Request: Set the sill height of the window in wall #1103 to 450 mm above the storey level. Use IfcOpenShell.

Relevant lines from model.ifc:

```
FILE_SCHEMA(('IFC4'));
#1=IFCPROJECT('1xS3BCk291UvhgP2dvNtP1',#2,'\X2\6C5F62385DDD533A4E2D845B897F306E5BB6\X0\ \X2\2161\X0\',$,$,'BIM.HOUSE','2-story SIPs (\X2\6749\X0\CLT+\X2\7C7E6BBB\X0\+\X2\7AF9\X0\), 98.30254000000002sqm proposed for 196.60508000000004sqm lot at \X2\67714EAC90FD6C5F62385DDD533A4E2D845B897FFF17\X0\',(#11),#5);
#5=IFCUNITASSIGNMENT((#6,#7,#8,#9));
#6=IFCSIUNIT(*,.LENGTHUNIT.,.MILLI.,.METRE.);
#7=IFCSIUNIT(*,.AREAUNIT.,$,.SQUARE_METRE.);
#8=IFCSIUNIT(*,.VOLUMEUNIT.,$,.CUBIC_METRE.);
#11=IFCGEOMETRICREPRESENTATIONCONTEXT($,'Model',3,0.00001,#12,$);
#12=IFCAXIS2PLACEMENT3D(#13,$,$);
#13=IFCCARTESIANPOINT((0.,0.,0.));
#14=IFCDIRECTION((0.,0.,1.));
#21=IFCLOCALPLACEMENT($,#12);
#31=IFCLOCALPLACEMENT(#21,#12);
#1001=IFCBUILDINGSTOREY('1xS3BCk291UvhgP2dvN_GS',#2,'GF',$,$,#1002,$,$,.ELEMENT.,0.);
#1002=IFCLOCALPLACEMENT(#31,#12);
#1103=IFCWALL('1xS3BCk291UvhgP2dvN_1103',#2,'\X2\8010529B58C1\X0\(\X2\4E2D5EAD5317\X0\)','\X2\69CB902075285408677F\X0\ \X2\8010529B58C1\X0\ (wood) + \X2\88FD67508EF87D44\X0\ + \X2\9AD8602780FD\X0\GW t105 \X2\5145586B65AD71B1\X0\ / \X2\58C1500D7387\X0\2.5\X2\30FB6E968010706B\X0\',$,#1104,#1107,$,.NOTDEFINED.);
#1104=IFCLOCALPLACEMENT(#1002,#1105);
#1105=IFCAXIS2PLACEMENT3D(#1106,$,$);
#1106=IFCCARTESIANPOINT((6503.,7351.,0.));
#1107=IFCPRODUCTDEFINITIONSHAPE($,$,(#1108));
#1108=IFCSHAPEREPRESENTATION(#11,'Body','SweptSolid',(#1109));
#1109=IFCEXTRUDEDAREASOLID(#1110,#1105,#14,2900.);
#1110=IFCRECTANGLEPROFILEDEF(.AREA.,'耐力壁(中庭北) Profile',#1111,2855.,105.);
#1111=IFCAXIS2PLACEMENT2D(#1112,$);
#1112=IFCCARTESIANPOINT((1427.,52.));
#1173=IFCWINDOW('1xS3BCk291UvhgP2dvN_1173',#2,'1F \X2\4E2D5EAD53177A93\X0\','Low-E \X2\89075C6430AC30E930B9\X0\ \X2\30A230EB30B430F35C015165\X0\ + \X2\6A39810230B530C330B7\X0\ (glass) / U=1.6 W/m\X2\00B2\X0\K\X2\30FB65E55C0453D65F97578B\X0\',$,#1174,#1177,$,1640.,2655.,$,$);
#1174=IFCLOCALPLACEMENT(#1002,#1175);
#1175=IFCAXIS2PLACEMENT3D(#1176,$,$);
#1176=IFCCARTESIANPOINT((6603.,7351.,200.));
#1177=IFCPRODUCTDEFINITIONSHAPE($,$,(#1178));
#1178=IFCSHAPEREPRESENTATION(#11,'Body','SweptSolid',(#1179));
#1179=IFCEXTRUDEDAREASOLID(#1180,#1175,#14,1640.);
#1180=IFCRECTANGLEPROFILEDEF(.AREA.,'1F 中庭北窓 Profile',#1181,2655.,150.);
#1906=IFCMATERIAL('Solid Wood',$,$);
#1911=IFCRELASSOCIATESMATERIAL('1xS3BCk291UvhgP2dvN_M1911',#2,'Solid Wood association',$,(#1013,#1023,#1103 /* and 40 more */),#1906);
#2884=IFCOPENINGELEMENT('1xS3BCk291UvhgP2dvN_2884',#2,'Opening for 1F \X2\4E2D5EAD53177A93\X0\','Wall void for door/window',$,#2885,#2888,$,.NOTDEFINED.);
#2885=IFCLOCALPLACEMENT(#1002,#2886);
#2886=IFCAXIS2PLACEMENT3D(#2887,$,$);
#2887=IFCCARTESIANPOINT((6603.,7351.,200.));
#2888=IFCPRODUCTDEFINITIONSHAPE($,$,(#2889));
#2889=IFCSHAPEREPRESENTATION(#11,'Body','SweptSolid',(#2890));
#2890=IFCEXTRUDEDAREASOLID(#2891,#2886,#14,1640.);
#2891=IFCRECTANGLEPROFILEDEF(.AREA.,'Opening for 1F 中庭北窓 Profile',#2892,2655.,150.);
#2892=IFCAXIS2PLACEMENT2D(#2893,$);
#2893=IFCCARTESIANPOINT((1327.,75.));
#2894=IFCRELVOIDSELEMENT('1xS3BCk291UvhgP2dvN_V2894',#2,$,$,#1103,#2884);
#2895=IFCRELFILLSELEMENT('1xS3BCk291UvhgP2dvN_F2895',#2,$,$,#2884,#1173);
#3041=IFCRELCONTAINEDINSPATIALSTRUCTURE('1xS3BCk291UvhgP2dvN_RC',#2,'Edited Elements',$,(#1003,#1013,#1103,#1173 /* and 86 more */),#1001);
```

```python
import numpy as np
import ifcopenshell
import ifcopenshell.api.geometry
import ifcopenshell.geom
import ifcopenshell.util.element
import ifcopenshell.util.placement
import ifcopenshell.util.shape
import ifcopenshell.util.unit

model = ifcopenshell.open("model.ifc")
unit_scale = ifcopenshell.util.unit.calculate_unit_scale(model)

window = model.by_guid("1xS3BCk291UvhgP2dvN_1173")
opening = window.FillsVoids[0].RelatingOpeningElement
storey = ifcopenshell.util.element.get_container(window, ifc_class="IfcBuildingStorey")
level = ifcopenshell.util.placement.get_local_placement(storey.ObjectPlacement)[2, 3]

# The opening's origin need not be at the sill, so measure its lowest point.
shape = ifcopenshell.geom.create_shape(ifcopenshell.geom.settings(), opening)
bottom = ifcopenshell.util.shape.get_shape_bottom_elevation(shape, shape.geometry) / unit_scale
dz = level + 0.45 / unit_scale - bottom

shift = np.array([0.0, 0.0, dz])
# The window is not placed relative to its opening, so move both.
for product in (opening, window):
    matrix = ifcopenshell.util.placement.get_local_placement(product.ObjectPlacement)
    matrix[:3, 3] += shift
    ifcopenshell.api.geometry.edit_object_placement(model, product=product, matrix=matrix, is_si=False)

print(f"moved by {dz * unit_scale:+.3f} m")

model.write("model_rev.ifc")
```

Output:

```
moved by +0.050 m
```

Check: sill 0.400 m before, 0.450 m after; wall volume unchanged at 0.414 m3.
